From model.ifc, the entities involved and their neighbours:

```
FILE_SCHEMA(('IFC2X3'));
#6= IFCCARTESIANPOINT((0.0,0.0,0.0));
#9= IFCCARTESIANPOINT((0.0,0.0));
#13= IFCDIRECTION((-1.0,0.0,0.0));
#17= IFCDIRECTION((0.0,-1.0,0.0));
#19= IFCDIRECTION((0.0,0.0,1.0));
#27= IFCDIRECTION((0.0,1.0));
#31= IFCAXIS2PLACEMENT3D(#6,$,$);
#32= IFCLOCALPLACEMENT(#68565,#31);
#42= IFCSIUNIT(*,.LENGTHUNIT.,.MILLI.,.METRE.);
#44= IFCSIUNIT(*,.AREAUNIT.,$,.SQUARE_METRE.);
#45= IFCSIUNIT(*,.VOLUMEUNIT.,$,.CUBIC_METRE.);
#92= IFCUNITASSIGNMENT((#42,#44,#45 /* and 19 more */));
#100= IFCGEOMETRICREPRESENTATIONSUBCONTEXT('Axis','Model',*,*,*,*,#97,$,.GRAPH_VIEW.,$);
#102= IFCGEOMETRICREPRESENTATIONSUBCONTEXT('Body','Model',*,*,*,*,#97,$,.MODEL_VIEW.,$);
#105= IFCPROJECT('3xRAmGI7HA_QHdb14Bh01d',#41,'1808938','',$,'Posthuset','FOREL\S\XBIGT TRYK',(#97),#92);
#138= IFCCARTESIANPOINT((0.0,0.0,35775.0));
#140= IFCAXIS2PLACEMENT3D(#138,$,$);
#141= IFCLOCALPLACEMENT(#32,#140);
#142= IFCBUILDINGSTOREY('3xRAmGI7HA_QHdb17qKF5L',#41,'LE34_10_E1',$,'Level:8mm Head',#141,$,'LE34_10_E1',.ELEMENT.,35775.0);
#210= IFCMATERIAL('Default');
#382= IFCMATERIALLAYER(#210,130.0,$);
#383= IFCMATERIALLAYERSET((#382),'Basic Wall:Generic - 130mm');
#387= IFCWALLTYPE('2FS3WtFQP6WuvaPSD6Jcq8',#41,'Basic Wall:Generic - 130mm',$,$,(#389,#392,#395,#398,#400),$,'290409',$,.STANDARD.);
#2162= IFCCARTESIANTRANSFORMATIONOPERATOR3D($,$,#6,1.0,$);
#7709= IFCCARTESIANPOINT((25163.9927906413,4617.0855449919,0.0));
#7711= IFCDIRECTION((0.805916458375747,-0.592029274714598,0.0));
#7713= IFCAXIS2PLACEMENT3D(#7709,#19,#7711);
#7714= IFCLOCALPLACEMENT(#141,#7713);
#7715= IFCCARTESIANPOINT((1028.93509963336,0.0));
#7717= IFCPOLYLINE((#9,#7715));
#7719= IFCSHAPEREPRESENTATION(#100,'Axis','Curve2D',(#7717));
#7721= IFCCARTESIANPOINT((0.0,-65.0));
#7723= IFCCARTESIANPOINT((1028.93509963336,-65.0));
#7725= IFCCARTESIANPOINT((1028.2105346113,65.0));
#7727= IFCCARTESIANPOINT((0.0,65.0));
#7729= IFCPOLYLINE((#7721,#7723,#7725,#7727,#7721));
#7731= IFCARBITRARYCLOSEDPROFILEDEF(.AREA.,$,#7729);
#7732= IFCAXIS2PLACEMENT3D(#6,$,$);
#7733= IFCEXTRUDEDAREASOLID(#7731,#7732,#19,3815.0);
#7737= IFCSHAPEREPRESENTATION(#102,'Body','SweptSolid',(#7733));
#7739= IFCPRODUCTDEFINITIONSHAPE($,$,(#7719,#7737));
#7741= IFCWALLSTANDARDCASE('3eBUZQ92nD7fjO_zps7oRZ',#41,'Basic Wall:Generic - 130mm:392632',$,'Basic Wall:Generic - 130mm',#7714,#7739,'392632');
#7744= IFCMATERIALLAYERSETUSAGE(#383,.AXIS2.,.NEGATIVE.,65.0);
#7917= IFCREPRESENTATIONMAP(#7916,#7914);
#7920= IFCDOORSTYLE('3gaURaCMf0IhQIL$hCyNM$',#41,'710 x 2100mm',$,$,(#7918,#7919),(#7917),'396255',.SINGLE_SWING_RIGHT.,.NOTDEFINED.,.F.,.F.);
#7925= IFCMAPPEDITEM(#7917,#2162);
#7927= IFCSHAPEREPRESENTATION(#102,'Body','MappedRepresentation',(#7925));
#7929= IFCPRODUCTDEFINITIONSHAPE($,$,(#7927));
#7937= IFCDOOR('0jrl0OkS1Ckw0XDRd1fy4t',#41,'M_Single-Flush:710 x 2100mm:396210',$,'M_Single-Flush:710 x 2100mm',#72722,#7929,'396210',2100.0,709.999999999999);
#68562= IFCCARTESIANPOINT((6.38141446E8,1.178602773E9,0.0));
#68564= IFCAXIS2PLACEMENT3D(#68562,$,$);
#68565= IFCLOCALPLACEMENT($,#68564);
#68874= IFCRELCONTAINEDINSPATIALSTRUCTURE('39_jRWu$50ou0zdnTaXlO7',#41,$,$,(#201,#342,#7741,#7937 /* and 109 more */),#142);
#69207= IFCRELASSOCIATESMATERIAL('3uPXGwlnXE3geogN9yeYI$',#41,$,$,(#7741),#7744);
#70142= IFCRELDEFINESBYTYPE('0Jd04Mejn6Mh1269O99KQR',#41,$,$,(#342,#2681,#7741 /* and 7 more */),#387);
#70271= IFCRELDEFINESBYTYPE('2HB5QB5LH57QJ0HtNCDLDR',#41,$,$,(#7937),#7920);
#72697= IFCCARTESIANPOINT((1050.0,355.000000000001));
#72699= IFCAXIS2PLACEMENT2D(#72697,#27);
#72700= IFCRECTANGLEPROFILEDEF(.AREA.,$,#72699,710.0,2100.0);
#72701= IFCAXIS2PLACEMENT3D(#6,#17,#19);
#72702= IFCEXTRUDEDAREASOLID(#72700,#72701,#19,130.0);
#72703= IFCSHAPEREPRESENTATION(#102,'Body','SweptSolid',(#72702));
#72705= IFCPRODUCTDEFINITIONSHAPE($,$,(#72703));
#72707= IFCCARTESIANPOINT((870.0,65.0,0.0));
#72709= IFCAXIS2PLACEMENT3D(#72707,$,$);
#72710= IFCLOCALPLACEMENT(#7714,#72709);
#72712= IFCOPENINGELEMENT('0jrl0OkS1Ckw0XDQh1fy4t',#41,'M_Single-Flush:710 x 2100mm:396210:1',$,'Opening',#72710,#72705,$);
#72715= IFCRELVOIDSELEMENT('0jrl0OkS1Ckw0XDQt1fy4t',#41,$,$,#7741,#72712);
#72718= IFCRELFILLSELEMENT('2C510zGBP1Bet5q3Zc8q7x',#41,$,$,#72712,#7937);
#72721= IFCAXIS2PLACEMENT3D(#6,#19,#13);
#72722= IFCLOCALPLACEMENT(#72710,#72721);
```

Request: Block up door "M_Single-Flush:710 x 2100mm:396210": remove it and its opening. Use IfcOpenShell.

```python
import ifcopenshell
import ifcopenshell.api.feature
import ifcopenshell.api.root
import ifcopenshell.geom
import ifcopenshell.util.shape

model = ifcopenshell.open("model.ifc")
settings = ifcopenshell.geom.settings()


def volume(element):
    """Net volume in cubic metres, openings subtracted."""
    shape = ifcopenshell.geom.create_shape(settings, element)
    return ifcopenshell.util.shape.get_volume(shape.geometry)


door = model.by_id(7937)
opening = door.FillsVoids[0].RelatingOpeningElement
wall = opening.VoidsElements[0].RelatingBuildingElement
before = volume(wall)

ifcopenshell.api.root.remove_product(model, product=door)
ifcopenshell.api.feature.remove_feature(model, feature=opening)

after = volume(wall)

print(f"wall volume {before:.3f} -> {after:.3f} m3")

model.write("model_updated.ifc")
```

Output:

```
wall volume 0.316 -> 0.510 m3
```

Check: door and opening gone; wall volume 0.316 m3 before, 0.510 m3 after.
